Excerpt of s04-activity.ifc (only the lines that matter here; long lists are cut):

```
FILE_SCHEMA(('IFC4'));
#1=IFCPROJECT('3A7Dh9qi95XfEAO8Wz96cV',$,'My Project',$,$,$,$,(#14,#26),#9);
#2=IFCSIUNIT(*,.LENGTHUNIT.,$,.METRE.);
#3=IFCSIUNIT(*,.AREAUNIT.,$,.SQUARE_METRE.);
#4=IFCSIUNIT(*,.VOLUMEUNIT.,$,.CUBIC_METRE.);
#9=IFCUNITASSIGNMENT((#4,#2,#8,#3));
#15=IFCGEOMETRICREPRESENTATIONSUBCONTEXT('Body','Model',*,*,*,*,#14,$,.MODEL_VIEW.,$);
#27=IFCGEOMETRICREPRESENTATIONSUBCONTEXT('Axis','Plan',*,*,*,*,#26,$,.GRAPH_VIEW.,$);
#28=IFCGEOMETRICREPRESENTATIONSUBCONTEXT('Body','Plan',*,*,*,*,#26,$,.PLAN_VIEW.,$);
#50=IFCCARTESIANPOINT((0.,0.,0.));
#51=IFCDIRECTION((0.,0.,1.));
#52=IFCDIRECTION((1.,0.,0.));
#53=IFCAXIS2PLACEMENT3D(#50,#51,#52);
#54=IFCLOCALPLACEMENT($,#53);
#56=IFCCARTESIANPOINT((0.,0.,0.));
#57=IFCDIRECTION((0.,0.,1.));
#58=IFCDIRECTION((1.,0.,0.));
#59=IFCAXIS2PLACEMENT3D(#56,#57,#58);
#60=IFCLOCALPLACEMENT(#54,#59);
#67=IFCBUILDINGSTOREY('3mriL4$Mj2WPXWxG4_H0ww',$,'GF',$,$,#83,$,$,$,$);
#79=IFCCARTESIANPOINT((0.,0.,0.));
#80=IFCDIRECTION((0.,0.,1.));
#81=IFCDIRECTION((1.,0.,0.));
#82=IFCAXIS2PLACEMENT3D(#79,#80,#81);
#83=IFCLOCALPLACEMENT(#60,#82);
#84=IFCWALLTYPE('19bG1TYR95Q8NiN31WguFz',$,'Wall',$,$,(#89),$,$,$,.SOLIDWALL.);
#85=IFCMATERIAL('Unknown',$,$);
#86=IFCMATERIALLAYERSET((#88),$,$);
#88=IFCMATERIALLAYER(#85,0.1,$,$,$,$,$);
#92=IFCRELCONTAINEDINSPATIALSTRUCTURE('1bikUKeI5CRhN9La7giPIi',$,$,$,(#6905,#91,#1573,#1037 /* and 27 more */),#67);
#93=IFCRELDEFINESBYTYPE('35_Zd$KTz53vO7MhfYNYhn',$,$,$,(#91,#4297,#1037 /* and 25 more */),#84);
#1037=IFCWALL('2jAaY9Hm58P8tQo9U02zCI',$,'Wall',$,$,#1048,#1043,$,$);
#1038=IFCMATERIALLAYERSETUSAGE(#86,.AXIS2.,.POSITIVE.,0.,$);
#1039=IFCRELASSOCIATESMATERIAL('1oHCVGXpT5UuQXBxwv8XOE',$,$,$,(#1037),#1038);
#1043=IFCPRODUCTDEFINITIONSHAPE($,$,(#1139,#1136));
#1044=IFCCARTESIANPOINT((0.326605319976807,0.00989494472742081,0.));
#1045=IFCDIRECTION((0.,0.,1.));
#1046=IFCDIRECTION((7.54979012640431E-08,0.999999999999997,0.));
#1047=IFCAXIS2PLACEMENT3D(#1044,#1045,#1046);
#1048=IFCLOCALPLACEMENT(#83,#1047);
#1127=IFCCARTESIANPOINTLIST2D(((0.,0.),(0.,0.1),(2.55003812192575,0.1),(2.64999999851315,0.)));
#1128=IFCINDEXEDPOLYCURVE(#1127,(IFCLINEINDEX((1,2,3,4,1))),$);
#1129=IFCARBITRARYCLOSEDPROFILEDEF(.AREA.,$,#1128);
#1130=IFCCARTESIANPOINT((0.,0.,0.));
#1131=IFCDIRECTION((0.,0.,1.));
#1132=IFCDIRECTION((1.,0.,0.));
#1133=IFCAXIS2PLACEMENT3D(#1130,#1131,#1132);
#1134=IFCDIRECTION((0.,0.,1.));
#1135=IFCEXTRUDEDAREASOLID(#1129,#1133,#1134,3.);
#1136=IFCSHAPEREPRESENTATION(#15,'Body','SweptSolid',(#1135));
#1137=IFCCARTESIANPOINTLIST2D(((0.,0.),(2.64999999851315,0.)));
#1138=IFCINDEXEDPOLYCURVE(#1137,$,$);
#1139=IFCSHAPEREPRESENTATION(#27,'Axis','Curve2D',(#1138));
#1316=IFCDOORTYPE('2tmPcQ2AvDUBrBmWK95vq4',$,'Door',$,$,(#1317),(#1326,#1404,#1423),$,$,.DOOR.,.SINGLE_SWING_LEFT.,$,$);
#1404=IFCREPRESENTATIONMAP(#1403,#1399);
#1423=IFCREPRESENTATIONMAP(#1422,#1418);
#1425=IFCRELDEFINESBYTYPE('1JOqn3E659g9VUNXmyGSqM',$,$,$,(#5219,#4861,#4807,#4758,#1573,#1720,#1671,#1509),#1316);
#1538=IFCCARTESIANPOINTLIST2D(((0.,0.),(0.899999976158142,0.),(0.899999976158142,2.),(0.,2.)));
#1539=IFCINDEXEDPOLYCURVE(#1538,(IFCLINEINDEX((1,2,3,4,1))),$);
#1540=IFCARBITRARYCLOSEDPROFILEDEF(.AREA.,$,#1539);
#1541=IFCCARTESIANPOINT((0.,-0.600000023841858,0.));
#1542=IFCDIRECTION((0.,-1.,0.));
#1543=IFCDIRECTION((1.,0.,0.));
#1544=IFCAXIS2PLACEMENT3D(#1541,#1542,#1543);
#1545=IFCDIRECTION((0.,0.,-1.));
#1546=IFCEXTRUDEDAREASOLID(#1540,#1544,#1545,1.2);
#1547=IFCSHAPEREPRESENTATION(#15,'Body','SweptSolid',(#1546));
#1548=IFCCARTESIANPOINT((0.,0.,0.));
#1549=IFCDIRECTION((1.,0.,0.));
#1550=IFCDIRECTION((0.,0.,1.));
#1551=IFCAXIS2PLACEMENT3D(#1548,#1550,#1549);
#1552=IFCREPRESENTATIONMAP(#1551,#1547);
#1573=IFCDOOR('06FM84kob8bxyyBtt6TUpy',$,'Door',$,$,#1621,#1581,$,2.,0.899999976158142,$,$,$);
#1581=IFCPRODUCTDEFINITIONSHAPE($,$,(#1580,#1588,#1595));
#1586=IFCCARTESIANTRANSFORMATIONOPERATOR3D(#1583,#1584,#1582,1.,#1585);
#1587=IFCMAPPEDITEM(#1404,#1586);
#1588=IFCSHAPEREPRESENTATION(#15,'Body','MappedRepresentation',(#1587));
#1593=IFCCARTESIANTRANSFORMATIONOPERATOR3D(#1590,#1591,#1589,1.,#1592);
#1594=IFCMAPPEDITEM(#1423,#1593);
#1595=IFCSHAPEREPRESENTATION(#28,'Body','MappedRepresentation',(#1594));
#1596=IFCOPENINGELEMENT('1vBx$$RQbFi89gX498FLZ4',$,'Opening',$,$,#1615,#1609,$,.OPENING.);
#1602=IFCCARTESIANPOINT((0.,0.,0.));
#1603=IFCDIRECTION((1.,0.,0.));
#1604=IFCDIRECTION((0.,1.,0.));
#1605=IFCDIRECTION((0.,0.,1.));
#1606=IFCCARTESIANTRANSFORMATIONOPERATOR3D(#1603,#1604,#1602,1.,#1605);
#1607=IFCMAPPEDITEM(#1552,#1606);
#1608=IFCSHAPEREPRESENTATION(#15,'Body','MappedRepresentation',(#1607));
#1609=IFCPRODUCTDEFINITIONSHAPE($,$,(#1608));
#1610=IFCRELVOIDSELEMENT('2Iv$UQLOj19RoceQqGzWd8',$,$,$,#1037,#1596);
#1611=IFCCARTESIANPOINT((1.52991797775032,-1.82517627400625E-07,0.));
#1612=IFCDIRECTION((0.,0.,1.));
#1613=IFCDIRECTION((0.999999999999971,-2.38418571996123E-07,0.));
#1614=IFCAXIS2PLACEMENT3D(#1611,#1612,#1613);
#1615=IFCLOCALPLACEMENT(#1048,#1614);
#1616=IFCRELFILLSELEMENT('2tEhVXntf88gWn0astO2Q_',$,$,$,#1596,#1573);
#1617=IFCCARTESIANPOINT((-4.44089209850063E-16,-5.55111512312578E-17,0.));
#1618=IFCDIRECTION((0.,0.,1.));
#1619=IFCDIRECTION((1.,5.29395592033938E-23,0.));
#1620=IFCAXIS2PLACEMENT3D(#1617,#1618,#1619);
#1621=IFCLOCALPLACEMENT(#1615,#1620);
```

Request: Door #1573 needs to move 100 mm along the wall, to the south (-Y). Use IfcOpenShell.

```python
import ifcopenshell
import ifcopenshell.api.geometry
import ifcopenshell.util.placement
import ifcopenshell.util.unit

model = ifcopenshell.open("s04-activity.ifc")
unit_scale = ifcopenshell.util.unit.calculate_unit_scale(model)

door = model.by_id(1573)
opening = door.FillsVoids[0].RelatingOpeningElement
wall = opening.VoidsElements[0].RelatingBuildingElement

wall_matrix = ifcopenshell.util.placement.get_local_placement(wall.ObjectPlacement)
shift = wall_matrix[:3, 0] * -0.1 / unit_scale
before = ifcopenshell.util.placement.get_local_placement(door.ObjectPlacement)[:3, 3].copy()

# The door is placed relative to its opening, so it follows when the opening moves.
matrix = ifcopenshell.util.placement.get_local_placement(opening.ObjectPlacement)
matrix[:3, 3] += shift
ifcopenshell.api.geometry.edit_object_placement(
    model, product=opening, matrix=matrix, is_si=False, should_transform_children=True
)

after = ifcopenshell.util.placement.get_local_placement(door.ObjectPlacement)[:3, 3]
print("door moved by", (after - before).round(3) + 0.0)

model.write("s04-activity_updated.ifc")
```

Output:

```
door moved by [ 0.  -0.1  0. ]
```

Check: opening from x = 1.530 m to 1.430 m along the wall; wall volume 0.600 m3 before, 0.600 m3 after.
